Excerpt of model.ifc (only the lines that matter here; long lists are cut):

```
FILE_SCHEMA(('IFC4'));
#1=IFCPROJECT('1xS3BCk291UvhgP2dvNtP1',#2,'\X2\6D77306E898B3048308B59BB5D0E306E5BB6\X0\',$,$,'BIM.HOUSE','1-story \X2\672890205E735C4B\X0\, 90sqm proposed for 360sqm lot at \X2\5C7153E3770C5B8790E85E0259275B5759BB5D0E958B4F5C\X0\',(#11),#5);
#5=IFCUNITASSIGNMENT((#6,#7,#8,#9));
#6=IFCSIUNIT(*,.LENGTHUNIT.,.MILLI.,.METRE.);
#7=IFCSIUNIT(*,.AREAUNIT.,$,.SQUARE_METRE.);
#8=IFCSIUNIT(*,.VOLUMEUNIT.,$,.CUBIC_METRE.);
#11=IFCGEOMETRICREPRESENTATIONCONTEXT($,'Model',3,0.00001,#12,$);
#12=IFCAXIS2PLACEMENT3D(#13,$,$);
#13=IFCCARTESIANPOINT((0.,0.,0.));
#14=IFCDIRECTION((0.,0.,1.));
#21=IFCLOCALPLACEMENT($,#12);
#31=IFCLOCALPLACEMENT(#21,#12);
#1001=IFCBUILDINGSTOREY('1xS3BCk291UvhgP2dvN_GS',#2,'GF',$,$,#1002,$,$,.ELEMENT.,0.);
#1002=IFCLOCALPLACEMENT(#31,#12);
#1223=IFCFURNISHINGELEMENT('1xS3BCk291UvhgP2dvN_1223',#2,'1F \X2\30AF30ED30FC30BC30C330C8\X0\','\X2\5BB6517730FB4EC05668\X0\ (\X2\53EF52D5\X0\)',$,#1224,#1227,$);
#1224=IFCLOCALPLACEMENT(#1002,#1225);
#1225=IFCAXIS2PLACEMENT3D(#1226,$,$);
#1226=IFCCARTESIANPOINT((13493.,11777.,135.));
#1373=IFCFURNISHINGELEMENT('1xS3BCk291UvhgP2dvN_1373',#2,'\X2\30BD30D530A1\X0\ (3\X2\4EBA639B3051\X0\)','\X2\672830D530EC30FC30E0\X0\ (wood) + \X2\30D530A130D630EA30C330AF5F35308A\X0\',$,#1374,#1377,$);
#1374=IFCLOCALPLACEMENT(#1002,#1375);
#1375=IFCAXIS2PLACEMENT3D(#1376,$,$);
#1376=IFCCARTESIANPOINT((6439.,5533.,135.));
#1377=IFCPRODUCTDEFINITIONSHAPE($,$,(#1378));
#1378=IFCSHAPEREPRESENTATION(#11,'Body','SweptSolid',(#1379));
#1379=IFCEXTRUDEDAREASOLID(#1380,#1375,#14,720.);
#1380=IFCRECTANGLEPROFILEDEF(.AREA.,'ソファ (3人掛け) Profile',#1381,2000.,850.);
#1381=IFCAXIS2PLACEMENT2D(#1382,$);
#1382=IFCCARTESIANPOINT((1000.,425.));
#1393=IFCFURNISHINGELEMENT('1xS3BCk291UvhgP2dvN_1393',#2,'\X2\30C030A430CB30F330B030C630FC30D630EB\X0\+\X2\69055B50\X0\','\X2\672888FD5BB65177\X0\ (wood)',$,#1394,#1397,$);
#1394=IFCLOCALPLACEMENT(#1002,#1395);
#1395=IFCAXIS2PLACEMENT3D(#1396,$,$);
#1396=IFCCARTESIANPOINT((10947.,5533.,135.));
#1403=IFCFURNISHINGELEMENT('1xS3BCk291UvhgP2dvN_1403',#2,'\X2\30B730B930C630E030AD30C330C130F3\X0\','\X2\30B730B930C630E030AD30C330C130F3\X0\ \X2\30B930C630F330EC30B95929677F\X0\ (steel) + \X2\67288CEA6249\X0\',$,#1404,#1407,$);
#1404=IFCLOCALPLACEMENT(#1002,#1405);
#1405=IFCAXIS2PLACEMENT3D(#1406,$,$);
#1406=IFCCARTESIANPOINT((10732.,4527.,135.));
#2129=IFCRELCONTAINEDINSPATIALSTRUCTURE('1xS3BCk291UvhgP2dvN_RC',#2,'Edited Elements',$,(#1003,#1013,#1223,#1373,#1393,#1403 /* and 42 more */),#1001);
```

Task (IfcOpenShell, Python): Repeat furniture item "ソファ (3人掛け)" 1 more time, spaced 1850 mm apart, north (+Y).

```python
import numpy as np
import ifcopenshell
import ifcopenshell.api.geometry
import ifcopenshell.api.root
import ifcopenshell.util.element
import ifcopenshell.util.placement

model = ifcopenshell.open("model.ifc")


def reuse_history(source, copy):
    """copy_class also copies each property set's owner history, people and application; keep the originals."""
    for rel in copy.IsDefinedBy:
        if rel.is_a("IfcRelDefinesByProperties") and (history := rel.RelatingPropertyDefinition.OwnerHistory):
            rel.RelatingPropertyDefinition.OwnerHistory = source.OwnerHistory
            ifcopenshell.util.element.remove_deep2(model, history)


source = model.by_guid("1xS3BCk291UvhgP2dvN_1373")
base = ifcopenshell.util.placement.get_local_placement(source.ObjectPlacement)
step = np.array([0.0, 1.0, 0.0]) * 1850.0

for i in range(1, 2):
    copy = ifcopenshell.api.root.copy_class(model, product=source)
    copy.Representation = ifcopenshell.util.element.copy_deep(
        model, source.Representation, exclude=["IfcGeometricRepresentationContext", "IfcRepresentationMap"]
    )
    reuse_history(source, copy)
    matrix = base.copy()
    matrix[:3, 3] += i * step
    print("added at", matrix[:3, 3].round(3) + 0.0)
    ifcopenshell.api.geometry.edit_object_placement(model, product=copy, matrix=matrix, is_si=False)

model.write("model_edited.ifc")
```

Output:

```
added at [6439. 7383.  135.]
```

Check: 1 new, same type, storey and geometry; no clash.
